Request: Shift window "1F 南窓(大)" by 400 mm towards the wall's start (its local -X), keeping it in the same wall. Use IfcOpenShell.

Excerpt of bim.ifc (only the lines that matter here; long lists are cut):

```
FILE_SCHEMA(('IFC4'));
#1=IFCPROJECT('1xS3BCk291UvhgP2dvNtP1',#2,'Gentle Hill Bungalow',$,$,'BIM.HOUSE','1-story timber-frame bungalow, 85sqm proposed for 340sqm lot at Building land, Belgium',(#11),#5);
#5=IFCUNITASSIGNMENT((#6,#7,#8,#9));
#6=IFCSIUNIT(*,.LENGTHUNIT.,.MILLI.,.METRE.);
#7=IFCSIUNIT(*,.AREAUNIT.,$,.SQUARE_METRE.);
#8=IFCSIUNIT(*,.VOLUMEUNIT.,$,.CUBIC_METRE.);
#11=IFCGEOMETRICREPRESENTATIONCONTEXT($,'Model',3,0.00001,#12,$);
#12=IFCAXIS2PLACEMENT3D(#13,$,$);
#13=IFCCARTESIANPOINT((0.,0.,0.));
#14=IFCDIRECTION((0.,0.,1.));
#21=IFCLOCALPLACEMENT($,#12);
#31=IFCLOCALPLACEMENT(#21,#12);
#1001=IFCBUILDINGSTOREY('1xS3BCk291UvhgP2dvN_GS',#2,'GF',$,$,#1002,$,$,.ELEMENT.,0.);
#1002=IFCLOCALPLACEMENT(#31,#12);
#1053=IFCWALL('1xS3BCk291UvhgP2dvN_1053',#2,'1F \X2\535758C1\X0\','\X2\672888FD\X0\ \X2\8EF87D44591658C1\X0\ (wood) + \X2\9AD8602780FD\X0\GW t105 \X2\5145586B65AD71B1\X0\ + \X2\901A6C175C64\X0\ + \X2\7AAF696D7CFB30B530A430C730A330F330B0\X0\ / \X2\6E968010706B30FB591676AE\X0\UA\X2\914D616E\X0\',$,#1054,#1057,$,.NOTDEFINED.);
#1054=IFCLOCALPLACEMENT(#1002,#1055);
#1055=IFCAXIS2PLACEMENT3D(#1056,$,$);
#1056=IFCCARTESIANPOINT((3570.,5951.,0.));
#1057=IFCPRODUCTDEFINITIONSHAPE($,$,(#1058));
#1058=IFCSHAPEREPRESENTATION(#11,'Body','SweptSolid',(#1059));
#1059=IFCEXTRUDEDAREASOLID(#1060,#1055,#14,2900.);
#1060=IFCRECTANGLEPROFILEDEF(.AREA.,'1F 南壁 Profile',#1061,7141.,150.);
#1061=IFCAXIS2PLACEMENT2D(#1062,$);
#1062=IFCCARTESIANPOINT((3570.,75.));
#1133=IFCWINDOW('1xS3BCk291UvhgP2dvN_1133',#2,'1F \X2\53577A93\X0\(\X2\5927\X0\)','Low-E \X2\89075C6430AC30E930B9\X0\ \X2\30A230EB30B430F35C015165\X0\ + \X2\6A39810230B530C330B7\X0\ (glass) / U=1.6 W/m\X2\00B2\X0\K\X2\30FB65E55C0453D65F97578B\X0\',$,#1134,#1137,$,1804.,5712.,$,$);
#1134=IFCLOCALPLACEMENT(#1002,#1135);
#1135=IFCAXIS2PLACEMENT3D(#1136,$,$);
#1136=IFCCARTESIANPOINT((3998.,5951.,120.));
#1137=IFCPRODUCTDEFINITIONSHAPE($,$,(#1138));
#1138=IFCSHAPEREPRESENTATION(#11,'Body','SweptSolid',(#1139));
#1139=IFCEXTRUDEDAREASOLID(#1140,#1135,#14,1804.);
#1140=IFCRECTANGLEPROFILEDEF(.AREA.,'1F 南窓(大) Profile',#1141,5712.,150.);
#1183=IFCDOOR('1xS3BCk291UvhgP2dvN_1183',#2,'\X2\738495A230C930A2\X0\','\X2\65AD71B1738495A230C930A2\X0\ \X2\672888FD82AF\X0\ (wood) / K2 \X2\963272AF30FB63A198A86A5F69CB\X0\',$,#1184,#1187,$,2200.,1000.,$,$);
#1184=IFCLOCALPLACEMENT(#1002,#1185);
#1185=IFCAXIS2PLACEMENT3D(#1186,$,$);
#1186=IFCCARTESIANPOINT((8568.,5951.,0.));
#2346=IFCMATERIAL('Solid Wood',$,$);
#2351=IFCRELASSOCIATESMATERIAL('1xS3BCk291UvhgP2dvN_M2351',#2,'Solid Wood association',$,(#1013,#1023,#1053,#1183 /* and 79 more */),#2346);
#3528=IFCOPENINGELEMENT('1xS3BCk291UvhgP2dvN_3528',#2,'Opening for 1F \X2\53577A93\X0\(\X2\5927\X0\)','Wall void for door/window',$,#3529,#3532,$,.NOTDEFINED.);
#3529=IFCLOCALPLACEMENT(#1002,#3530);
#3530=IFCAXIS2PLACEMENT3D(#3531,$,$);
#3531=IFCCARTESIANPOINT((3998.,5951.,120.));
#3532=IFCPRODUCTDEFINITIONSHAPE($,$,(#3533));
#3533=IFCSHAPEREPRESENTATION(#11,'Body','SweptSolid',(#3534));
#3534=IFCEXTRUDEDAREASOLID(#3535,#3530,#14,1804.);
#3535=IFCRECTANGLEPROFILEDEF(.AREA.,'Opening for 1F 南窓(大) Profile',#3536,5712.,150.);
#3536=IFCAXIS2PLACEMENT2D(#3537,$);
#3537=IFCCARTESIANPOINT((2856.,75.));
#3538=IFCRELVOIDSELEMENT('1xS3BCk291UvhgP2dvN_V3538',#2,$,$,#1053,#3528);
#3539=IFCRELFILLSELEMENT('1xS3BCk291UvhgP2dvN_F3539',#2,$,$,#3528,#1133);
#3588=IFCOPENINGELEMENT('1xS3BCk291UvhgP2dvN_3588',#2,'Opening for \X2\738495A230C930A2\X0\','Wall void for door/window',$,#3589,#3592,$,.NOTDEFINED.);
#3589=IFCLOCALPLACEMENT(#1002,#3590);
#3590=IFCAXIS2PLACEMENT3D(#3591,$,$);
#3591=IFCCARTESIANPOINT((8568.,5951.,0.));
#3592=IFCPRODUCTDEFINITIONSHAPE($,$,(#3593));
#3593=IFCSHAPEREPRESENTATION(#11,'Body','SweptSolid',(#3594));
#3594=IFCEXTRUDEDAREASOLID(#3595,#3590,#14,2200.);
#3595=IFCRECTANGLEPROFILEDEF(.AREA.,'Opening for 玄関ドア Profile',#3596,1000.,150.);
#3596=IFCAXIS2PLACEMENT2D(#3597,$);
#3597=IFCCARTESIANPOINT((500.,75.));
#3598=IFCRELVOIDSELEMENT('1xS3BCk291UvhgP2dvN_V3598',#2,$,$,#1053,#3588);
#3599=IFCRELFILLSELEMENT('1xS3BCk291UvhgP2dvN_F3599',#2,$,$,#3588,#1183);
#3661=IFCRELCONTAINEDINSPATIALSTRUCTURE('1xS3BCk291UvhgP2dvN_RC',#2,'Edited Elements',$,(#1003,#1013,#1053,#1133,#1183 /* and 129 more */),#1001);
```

```python
import ifcopenshell
import ifcopenshell.api.geometry
import ifcopenshell.util.placement

model = ifcopenshell.open("bim.ifc")

window = model.by_guid("1xS3BCk291UvhgP2dvN_1133")
opening = window.FillsVoids[0].RelatingOpeningElement
wall = opening.VoidsElements[0].RelatingBuildingElement

wall_matrix = ifcopenshell.util.placement.get_local_placement(wall.ObjectPlacement)
shift = wall_matrix[:3, 0] * -400.0
before = ifcopenshell.util.placement.get_local_placement(window.ObjectPlacement)[:3, 3].copy()

# The window is not placed relative to its opening, so move both.
for product in (opening, window):
    matrix = ifcopenshell.util.placement.get_local_placement(product.ObjectPlacement)
    matrix[:3, 3] += shift
    ifcopenshell.api.geometry.edit_object_placement(model, product=product, matrix=matrix, is_si=False)

after = ifcopenshell.util.placement.get_local_placement(window.ObjectPlacement)[:3, 3]
print("window moved by", (after - before).round(3) + 0.0)

model.write("bim_v2.ifc")
```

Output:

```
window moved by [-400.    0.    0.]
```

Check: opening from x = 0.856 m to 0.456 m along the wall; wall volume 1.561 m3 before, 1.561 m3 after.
